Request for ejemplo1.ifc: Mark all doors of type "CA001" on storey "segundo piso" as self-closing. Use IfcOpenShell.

First a look at what the model holds.

```python
import ifcopenshell
import ifcopenshell.util.element

model = ifcopenshell.open("ejemplo1.ifc")
print(model.schema)
storey = next(s for s in model.by_type("IfcBuildingStorey") if s.Name == "segundo piso")
doors = [e for e in ifcopenshell.util.element.get_decomposition(storey) if e.is_a("IfcDoor")]
seen = {}
for e in doors:
    element_type = ifcopenshell.util.element.get_type(e)
    key = (element_type.Name if element_type != e and element_type else None, ifcopenshell.util.element.get_pset(e, "Pset_DoorCommon", "SelfClosing"))
    seen[key] = seen.get(key, 0) + 1
for (name, value), count in sorted(seen.items(), key=str):
    print(count, "x", name, "|", value)
```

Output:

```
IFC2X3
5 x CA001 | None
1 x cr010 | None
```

```python
import ifcopenshell
import ifcopenshell.api.pset
import ifcopenshell.util.element

model = ifcopenshell.open("ejemplo1.ifc")

storey = next(s for s in model.by_type("IfcBuildingStorey") if s.Name == "segundo piso")
doors = [e for e in ifcopenshell.util.element.get_decomposition(storey) if e.is_a("IfcDoor")]

count = 0
for e in doors:
    element_type = ifcopenshell.util.element.get_type(e)
    if element_type in (None, e) or element_type.Name != "CA001":
        continue
    # add_pset returns the element's existing set when there is one.
    pset = ifcopenshell.api.pset.add_pset(model, product=e, name="Pset_DoorCommon")
    ifcopenshell.api.pset.edit_pset(model, pset=pset, properties={"SelfClosing": True})
    count += 1

print(count, "doors updated")

model.write("ejemplo1_edited.ifc")
```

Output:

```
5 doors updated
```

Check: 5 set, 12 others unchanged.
